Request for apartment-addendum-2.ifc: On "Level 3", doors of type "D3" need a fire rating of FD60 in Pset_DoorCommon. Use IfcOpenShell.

First a look at what the model holds.

```python
import ifcopenshell
import ifcopenshell.util.element

model = ifcopenshell.open("apartment-addendum-2.ifc")
print(model.schema)
storey = next(s for s in model.by_type("IfcBuildingStorey") if s.Name == "Level 3")
doors = [e for e in ifcopenshell.util.element.get_decomposition(storey) if e.is_a("IfcDoor")]
seen = {}
for e in doors:
    element_type = ifcopenshell.util.element.get_type(e)
    key = (element_type.Name if element_type != e and element_type else None, ifcopenshell.util.element.get_pset(e, "Pset_DoorCommon", "FireRating"))
    seen[key] = seen.get(key, 0) + 1
for (name, value), count in sorted(seen.items(), key=str):
    print(count, "x", name, "|", value)
```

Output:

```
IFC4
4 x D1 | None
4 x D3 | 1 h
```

```python
import ifcopenshell
import ifcopenshell.api.pset
import ifcopenshell.util.element

model = ifcopenshell.open("apartment-addendum-2.ifc")

storey = next(s for s in model.by_type("IfcBuildingStorey") if s.Name == "Level 3")
doors = [e for e in ifcopenshell.util.element.get_decomposition(storey) if e.is_a("IfcDoor")]

count = 0
for e in doors:
    element_type = ifcopenshell.util.element.get_type(e)
    if element_type in (None, e) or element_type.Name != "D3":
        continue
    # add_pset returns the element's existing set when there is one.
    pset = ifcopenshell.api.pset.add_pset(model, product=e, name="Pset_DoorCommon")
    ifcopenshell.api.pset.edit_pset(model, pset=pset, properties={"FireRating": "FD60"})
    count += 1

print(count, "doors updated")

model.write("apartment-addendum-2_updated.ifc")
```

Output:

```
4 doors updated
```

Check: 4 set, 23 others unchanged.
